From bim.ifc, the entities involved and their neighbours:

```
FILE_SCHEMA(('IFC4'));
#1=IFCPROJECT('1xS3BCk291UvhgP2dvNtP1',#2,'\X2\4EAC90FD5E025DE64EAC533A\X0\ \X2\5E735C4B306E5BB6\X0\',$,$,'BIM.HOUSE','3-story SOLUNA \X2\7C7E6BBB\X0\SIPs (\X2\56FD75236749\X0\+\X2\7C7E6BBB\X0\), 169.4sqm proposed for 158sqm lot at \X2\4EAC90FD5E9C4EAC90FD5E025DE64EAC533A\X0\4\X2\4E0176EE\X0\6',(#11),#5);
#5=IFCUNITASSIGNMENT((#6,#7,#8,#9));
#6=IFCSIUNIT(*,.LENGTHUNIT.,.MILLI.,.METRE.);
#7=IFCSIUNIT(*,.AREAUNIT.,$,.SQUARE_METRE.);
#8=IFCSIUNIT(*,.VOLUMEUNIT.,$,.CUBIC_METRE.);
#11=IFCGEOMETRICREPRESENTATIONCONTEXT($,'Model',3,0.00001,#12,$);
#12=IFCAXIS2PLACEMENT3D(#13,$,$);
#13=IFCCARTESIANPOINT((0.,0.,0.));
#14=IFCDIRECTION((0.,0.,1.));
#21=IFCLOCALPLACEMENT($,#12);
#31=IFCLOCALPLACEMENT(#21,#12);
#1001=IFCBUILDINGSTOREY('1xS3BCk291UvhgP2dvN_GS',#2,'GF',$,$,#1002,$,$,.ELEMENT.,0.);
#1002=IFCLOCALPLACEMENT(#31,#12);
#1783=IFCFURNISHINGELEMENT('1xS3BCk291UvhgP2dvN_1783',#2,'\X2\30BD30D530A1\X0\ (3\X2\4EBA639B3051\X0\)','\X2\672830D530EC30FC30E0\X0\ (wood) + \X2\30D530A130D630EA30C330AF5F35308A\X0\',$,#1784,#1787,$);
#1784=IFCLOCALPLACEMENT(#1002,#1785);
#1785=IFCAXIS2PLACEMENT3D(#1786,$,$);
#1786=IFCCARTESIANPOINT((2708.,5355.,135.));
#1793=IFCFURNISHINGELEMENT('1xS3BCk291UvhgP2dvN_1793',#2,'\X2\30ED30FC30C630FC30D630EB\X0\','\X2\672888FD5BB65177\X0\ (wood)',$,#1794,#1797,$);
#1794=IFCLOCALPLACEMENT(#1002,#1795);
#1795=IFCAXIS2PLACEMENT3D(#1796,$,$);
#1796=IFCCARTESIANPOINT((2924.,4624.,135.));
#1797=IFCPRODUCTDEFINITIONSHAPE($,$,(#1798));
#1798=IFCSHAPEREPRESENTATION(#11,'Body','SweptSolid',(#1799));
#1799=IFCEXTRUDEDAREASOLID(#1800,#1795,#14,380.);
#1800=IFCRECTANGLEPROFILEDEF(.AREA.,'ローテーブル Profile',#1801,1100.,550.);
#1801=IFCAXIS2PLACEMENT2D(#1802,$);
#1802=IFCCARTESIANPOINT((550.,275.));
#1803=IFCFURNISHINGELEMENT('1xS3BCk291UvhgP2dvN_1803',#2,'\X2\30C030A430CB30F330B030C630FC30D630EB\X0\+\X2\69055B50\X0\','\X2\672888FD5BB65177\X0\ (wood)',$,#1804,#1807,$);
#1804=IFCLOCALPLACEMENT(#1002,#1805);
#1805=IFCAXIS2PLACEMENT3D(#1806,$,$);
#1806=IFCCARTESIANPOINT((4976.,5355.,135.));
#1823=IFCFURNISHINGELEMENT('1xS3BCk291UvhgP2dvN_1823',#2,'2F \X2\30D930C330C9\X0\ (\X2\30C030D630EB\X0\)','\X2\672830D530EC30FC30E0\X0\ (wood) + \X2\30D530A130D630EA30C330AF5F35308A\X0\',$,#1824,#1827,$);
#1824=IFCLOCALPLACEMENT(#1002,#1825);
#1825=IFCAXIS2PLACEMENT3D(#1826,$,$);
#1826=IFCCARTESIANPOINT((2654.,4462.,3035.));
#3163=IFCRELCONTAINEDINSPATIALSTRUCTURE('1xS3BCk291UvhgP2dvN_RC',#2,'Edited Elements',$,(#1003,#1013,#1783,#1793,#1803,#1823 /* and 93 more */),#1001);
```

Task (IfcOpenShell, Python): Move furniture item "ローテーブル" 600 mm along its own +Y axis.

```python
import ifcopenshell
import ifcopenshell.api.geometry
import ifcopenshell.util.placement
import ifcopenshell.util.unit

model = ifcopenshell.open("bim.ifc")
unit_scale = ifcopenshell.util.unit.calculate_unit_scale(model)

item = model.by_guid("1xS3BCk291UvhgP2dvN_1793")
matrix = ifcopenshell.util.placement.get_local_placement(item.ObjectPlacement)
matrix[:3, 3] += matrix[:3, 1] * 0.6 / unit_scale
ifcopenshell.api.geometry.edit_object_placement(model, product=item, matrix=matrix, is_si=False)

print(ifcopenshell.util.placement.get_local_placement(item.ObjectPlacement).round(3) + 0.0)

model.write("bim_v2.ifc")
```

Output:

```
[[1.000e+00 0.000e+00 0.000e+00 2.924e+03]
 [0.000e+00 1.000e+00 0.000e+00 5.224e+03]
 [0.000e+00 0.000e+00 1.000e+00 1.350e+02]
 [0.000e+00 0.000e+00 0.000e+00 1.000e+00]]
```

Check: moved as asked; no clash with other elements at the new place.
